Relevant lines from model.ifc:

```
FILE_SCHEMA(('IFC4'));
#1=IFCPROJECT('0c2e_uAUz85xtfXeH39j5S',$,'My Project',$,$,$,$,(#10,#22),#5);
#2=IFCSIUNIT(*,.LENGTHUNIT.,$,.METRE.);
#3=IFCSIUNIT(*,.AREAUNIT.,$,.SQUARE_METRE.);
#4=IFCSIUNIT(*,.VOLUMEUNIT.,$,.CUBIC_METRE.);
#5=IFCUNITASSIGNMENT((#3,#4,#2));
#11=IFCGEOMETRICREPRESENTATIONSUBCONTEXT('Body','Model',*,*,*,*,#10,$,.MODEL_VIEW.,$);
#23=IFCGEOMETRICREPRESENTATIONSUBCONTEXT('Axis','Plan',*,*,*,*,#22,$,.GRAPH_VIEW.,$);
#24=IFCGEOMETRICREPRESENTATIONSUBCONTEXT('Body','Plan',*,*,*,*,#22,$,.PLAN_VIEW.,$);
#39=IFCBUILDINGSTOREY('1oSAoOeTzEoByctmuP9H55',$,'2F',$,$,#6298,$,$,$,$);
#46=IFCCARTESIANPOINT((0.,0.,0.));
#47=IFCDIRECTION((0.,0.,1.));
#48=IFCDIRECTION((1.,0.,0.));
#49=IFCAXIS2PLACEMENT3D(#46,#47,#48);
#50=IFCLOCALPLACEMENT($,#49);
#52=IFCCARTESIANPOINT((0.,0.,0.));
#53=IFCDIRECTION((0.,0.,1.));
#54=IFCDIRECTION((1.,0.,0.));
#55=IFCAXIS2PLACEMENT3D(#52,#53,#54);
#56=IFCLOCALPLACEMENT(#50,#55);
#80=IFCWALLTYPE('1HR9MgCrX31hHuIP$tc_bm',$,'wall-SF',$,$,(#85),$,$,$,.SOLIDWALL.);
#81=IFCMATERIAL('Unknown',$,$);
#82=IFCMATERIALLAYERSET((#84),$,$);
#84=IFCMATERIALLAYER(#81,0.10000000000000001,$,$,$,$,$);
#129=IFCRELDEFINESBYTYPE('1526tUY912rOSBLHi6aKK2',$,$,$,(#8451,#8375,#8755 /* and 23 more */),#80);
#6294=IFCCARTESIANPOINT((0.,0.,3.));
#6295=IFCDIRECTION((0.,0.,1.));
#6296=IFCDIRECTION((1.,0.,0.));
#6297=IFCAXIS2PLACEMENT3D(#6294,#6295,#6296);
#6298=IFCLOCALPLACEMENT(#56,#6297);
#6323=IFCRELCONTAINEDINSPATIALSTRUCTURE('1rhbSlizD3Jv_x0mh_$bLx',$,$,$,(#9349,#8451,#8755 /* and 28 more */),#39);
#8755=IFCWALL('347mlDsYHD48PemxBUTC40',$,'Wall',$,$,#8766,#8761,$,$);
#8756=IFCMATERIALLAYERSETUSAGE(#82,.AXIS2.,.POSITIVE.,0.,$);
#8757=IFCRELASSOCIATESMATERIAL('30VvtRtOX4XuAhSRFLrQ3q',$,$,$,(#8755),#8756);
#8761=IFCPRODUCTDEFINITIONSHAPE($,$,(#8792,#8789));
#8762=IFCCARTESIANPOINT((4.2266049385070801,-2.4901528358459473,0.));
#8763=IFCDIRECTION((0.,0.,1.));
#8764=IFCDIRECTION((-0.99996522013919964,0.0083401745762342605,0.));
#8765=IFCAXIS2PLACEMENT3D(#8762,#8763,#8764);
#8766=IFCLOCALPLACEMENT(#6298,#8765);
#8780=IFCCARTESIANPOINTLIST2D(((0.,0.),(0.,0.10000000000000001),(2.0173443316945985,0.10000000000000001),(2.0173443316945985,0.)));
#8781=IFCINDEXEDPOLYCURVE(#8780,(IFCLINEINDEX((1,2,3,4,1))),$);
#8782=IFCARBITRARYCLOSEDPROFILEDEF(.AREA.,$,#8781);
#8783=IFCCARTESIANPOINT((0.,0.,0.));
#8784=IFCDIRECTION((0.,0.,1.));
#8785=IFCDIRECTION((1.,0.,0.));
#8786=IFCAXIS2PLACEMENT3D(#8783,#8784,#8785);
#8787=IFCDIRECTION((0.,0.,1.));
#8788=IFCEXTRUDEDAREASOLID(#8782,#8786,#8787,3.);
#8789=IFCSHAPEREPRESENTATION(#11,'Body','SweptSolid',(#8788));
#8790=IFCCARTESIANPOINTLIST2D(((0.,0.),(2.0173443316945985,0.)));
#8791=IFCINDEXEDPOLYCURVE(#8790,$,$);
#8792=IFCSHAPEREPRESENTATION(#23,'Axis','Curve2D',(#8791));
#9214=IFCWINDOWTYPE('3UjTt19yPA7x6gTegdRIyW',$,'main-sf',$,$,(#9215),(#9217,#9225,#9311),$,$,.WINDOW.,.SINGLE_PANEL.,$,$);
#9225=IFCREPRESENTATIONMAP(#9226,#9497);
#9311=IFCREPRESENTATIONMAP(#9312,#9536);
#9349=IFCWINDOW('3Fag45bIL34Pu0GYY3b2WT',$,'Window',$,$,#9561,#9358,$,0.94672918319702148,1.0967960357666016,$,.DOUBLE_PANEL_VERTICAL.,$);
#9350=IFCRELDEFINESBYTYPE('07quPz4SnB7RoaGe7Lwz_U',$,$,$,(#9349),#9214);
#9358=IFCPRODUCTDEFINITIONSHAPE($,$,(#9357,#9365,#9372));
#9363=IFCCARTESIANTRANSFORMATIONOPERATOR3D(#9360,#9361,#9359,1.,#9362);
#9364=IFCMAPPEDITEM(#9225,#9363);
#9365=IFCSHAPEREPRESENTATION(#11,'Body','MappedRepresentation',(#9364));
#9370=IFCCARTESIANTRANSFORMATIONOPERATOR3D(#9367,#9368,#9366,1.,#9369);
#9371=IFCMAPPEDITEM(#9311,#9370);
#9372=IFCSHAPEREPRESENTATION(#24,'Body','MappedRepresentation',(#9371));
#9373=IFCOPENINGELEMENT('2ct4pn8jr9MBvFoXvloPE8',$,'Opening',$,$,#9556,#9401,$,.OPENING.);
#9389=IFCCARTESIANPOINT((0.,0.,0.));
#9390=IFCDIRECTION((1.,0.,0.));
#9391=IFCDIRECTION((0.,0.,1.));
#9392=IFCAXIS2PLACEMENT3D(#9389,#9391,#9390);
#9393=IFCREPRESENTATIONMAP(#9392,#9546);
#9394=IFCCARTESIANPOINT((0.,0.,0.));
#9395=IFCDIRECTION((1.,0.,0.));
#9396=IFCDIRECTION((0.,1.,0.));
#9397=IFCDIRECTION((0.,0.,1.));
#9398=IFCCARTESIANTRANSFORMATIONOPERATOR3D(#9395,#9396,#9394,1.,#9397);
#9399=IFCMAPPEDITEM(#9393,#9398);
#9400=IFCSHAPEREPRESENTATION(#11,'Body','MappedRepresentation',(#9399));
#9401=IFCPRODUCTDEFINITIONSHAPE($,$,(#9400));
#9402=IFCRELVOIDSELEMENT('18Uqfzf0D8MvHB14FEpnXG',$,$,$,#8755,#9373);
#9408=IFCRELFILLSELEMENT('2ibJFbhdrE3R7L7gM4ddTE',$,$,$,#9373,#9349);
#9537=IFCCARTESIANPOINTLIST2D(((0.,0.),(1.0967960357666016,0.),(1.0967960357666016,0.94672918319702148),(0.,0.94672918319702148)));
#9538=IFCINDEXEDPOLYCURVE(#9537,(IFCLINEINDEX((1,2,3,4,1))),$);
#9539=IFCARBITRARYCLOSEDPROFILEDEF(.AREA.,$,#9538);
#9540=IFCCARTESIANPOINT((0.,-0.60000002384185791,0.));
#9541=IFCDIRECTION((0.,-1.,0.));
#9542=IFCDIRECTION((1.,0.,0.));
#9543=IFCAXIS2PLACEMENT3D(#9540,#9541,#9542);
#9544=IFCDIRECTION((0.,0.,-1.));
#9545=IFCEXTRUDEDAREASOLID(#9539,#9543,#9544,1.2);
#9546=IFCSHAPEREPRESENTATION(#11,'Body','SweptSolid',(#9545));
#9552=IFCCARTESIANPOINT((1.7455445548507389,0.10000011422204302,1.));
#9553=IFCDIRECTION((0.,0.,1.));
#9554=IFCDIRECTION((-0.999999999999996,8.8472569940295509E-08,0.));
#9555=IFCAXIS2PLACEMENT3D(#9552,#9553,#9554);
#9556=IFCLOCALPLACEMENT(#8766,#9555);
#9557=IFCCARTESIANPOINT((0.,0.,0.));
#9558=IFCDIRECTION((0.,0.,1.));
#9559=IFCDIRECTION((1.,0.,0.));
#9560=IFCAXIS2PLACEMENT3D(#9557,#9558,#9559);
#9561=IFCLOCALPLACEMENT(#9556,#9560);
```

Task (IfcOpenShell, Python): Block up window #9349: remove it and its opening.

```python
import ifcopenshell
import ifcopenshell.api.feature
import ifcopenshell.api.root
import ifcopenshell.geom
import ifcopenshell.util.shape

model = ifcopenshell.open("model.ifc")
settings = ifcopenshell.geom.settings()


def volume(element):
    """Net volume in cubic metres, openings subtracted."""
    shape = ifcopenshell.geom.create_shape(settings, element)
    return ifcopenshell.util.shape.get_volume(shape.geometry)


window = model.by_guid("3Fag45bIL34Pu0GYY3b2WT")
opening = window.FillsVoids[0].RelatingOpeningElement
wall = opening.VoidsElements[0].RelatingBuildingElement
before = volume(wall)

ifcopenshell.api.root.remove_product(model, product=window)
ifcopenshell.api.feature.remove_feature(model, feature=opening)

after = volume(wall)

print(f"wall volume {before:.3f} -> {after:.3f} m3")

model.write("model_edited.ifc")
```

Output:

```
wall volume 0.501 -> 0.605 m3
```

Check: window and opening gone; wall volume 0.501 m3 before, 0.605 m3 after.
